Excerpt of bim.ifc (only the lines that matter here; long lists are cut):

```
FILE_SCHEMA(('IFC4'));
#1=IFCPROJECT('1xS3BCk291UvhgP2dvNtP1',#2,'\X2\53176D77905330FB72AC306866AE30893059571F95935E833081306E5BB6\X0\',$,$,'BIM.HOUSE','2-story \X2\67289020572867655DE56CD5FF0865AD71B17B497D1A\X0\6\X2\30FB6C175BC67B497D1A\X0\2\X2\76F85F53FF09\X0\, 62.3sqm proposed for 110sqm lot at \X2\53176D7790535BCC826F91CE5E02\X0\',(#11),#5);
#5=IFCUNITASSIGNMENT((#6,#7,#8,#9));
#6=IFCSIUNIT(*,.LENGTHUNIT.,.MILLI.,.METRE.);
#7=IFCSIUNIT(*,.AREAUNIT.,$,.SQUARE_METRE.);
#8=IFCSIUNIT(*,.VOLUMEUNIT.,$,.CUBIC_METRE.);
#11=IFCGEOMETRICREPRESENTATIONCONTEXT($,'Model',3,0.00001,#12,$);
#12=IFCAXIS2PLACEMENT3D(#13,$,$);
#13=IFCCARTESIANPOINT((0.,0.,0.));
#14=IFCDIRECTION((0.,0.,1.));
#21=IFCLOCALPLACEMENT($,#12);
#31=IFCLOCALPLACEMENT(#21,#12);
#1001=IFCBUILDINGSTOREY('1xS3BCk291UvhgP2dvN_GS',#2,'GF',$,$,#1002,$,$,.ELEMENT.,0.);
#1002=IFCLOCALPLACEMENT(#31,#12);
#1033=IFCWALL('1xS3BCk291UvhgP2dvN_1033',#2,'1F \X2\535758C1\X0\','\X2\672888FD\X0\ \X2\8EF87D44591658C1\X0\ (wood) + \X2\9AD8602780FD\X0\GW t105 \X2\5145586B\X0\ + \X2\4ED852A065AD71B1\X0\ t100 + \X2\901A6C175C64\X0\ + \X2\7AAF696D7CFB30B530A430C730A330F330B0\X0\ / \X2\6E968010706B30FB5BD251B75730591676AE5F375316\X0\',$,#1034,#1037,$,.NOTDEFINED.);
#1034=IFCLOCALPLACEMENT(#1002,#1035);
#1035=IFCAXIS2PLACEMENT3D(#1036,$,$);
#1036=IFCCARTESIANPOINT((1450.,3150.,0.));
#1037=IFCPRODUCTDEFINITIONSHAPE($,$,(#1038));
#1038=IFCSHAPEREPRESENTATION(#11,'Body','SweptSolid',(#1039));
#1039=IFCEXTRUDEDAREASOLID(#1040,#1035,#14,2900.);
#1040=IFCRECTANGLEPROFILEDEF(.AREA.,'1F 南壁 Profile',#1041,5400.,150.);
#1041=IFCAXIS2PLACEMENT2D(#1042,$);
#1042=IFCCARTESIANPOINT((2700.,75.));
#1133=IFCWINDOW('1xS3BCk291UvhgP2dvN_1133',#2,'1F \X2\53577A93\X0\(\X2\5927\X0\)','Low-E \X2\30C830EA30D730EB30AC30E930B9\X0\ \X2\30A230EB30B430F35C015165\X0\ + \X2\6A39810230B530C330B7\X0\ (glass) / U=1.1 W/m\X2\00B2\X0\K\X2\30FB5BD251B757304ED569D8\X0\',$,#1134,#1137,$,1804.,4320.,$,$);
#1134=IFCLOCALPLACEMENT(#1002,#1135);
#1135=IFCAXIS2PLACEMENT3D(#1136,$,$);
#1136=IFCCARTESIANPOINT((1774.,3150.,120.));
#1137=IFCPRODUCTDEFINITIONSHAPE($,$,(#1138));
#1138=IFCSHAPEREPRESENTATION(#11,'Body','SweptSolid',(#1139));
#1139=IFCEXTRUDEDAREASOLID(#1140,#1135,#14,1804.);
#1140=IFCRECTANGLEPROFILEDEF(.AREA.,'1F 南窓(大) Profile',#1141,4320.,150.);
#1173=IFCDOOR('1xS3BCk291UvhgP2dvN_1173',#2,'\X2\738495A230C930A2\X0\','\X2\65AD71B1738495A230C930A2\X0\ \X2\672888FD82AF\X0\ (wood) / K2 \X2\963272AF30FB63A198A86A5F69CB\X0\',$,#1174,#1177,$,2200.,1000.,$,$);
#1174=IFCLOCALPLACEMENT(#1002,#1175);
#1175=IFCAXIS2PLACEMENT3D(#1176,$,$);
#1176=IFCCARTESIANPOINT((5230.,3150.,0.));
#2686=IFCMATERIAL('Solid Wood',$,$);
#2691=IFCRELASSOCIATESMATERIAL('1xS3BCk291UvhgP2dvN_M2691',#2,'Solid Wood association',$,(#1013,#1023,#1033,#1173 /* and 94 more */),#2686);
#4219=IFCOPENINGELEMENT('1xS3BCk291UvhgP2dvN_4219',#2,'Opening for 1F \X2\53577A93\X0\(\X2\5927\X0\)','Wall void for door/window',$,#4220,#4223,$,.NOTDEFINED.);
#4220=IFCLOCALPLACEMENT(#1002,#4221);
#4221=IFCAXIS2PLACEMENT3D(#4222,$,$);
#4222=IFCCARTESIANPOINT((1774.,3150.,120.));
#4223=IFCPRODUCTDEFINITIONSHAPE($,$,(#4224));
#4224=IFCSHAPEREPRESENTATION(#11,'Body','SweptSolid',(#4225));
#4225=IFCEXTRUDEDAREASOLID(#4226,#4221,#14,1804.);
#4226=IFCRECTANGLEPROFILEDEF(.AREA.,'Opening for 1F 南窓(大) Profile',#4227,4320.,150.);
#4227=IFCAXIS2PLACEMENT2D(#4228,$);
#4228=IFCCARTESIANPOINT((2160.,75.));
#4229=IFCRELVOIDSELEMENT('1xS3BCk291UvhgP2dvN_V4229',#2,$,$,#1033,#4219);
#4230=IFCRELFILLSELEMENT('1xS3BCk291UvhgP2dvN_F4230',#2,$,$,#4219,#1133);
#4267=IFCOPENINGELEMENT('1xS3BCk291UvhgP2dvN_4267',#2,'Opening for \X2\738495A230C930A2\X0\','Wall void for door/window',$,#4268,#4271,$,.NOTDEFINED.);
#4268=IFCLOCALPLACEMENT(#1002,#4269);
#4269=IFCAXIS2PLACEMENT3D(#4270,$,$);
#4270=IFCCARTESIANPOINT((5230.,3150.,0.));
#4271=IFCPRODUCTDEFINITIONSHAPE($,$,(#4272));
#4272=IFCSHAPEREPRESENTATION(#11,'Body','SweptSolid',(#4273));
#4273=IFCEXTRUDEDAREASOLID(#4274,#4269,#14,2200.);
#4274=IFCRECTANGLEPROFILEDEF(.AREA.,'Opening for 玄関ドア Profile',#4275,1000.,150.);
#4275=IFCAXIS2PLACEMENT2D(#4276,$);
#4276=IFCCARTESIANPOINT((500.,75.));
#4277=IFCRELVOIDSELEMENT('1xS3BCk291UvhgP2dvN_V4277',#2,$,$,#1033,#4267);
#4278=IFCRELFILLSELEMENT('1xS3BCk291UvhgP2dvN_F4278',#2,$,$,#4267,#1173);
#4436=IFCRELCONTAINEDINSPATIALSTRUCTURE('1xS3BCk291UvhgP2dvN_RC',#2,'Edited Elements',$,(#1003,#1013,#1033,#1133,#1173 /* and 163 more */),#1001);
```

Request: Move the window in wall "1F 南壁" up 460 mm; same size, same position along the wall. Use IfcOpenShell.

```python
import numpy as np
import ifcopenshell
import ifcopenshell.api.geometry
import ifcopenshell.util.placement
import ifcopenshell.util.unit

model = ifcopenshell.open("bim.ifc")
unit_scale = ifcopenshell.util.unit.calculate_unit_scale(model)

window = model.by_id(1133)
opening = window.FillsVoids[0].RelatingOpeningElement
dz = 0.46 / unit_scale

shift = np.array([0.0, 0.0, dz])
# The window is not placed relative to its opening, so move both.
for product in (opening, window):
    matrix = ifcopenshell.util.placement.get_local_placement(product.ObjectPlacement)
    matrix[:3, 3] += shift
    ifcopenshell.api.geometry.edit_object_placement(model, product=product, matrix=matrix, is_si=False)

print(f"moved by {dz * unit_scale:+.3f} m")

model.write("bim_v2.ifc")
```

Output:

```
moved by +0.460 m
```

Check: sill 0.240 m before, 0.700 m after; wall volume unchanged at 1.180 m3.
